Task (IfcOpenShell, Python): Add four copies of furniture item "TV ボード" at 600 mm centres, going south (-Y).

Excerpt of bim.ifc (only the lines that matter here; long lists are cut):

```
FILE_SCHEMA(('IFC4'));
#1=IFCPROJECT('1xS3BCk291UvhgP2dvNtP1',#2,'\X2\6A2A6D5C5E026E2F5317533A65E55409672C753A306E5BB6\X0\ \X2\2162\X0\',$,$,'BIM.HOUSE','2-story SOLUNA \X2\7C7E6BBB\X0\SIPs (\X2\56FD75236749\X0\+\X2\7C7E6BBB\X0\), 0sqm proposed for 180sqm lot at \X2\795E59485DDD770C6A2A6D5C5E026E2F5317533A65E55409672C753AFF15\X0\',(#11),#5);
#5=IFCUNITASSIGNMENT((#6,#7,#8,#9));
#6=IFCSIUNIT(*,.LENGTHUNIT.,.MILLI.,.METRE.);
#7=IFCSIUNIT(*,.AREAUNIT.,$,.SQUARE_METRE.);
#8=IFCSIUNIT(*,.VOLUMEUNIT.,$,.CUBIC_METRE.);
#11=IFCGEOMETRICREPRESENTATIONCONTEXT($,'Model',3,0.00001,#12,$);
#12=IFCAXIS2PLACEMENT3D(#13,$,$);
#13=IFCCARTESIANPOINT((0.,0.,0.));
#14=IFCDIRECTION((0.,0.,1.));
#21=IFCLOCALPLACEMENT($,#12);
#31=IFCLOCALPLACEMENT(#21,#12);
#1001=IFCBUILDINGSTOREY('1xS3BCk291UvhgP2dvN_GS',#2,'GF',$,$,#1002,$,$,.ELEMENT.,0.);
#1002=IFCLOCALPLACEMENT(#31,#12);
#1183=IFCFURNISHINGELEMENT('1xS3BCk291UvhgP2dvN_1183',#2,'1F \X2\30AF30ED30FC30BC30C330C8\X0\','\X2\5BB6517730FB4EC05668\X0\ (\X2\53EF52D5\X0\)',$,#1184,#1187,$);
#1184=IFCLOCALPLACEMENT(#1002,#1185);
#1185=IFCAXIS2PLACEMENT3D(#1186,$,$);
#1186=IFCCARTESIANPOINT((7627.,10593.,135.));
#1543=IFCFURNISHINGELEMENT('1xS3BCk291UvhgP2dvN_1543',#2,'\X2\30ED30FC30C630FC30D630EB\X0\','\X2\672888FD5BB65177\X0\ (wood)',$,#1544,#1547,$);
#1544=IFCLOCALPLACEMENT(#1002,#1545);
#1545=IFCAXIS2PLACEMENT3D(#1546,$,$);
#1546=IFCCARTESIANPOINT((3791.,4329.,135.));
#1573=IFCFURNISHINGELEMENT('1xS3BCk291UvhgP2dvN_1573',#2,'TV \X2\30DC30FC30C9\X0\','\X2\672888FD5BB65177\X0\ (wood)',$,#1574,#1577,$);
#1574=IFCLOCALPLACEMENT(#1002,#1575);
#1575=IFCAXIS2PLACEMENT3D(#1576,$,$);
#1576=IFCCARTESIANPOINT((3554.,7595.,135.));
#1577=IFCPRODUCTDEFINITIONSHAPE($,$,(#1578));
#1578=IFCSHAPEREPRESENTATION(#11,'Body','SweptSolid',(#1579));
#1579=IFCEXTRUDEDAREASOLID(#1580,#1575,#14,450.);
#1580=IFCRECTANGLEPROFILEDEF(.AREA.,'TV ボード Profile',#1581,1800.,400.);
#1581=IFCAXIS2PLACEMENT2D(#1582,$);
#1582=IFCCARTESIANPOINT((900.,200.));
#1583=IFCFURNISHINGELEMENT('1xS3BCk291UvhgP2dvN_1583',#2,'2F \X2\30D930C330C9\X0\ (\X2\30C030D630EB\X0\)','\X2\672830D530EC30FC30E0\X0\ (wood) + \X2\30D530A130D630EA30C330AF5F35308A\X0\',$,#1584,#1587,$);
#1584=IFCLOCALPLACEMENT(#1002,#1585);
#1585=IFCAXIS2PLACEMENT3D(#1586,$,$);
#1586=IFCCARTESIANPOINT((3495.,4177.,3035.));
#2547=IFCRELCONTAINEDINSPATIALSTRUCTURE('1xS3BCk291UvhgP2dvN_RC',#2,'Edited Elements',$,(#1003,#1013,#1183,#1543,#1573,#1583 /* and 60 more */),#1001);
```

```python
import numpy as np
import ifcopenshell
import ifcopenshell.api.geometry
import ifcopenshell.api.root
import ifcopenshell.util.element
import ifcopenshell.util.placement
import ifcopenshell.util.unit

model = ifcopenshell.open("bim.ifc")
unit_scale = ifcopenshell.util.unit.calculate_unit_scale(model)


def reuse_history(source, copy):
    """copy_class also copies each property set's owner history, people and application; keep the originals."""
    for rel in copy.IsDefinedBy:
        if rel.is_a("IfcRelDefinesByProperties") and (history := rel.RelatingPropertyDefinition.OwnerHistory):
            rel.RelatingPropertyDefinition.OwnerHistory = source.OwnerHistory
            ifcopenshell.util.element.remove_deep2(model, history)


source = model.by_guid("1xS3BCk291UvhgP2dvN_1573")
base = ifcopenshell.util.placement.get_local_placement(source.ObjectPlacement)
step = np.array([0.0, -1.0, 0.0]) * 0.6 / unit_scale

for i in range(1, 5):
    copy = ifcopenshell.api.root.copy_class(model, product=source)
    copy.Representation = ifcopenshell.util.element.copy_deep(
        model, source.Representation, exclude=["IfcGeometricRepresentationContext", "IfcRepresentationMap"]
    )
    reuse_history(source, copy)
    matrix = base.copy()
    matrix[:3, 3] += i * step
    print("added at", matrix[:3, 3].round(3) + 0.0)
    ifcopenshell.api.geometry.edit_object_placement(model, product=copy, matrix=matrix, is_si=False)

model.write("bim-out.ifc")
```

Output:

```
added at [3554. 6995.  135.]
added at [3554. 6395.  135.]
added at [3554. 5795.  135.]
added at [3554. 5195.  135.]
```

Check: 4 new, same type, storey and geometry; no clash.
